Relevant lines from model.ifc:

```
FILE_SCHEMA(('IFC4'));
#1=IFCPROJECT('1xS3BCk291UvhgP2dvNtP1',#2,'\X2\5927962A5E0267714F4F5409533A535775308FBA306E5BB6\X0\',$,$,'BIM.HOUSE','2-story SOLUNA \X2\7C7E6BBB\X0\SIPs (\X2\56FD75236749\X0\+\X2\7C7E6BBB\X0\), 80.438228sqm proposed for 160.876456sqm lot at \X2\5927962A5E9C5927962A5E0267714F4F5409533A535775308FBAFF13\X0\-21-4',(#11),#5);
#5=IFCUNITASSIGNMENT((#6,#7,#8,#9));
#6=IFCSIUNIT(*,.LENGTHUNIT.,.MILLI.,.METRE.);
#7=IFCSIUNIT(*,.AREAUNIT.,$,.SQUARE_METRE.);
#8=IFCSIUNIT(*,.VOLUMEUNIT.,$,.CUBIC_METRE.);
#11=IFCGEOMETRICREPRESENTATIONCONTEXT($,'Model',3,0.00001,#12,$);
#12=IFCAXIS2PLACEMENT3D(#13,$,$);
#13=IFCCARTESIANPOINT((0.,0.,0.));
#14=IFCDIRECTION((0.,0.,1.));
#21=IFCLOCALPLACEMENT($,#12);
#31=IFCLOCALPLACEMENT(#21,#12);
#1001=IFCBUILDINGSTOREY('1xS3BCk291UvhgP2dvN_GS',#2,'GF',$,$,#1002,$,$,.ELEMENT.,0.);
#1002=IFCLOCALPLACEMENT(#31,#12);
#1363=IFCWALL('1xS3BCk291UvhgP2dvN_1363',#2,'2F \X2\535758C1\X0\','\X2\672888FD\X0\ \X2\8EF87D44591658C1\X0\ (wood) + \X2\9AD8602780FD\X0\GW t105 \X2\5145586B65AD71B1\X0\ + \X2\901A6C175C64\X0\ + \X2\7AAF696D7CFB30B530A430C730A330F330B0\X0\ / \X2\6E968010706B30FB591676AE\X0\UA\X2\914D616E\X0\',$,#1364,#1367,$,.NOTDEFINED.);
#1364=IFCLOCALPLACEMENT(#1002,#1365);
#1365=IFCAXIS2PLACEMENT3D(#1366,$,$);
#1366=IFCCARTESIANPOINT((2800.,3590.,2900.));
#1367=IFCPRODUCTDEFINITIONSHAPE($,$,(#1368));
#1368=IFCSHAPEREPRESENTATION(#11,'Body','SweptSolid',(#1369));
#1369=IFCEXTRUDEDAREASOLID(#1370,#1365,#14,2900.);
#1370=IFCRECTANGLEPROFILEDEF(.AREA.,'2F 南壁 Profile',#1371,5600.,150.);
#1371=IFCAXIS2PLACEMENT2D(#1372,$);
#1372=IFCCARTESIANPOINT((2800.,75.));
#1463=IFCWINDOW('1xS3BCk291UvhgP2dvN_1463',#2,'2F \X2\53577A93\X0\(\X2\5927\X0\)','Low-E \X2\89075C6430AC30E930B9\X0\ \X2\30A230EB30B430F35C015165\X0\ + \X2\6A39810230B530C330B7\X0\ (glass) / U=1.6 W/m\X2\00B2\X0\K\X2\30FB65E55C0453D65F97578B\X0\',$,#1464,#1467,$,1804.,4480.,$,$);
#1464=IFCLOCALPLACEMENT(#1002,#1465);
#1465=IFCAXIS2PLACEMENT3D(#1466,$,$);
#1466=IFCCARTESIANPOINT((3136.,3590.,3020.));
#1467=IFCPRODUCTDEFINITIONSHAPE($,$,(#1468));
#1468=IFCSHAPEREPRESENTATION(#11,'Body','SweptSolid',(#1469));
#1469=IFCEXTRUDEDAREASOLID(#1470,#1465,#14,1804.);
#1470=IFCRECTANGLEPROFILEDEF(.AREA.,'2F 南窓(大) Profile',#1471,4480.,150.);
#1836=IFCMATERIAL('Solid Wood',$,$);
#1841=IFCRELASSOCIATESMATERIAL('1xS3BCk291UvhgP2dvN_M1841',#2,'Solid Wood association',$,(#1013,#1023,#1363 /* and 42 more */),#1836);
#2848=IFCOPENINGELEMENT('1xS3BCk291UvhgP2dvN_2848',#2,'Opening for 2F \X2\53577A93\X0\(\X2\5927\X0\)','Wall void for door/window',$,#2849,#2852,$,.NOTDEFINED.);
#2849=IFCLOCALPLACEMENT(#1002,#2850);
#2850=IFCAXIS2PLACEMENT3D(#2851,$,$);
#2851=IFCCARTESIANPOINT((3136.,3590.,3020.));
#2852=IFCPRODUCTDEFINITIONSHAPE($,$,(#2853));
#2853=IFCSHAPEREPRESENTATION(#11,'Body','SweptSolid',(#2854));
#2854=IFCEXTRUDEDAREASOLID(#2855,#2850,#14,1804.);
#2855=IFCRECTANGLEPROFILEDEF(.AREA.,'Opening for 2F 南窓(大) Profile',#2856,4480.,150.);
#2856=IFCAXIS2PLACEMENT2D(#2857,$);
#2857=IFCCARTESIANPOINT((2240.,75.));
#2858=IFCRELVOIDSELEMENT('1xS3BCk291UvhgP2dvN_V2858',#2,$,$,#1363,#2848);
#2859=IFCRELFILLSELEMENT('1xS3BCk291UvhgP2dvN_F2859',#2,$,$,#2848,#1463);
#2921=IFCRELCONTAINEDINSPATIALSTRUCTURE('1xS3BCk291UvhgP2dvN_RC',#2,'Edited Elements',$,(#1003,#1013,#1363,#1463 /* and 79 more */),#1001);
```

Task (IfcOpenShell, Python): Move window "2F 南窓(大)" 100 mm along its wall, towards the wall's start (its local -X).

```python
import ifcopenshell
import ifcopenshell.api.geometry
import ifcopenshell.util.placement
import ifcopenshell.util.unit

model = ifcopenshell.open("model.ifc")
unit_scale = ifcopenshell.util.unit.calculate_unit_scale(model)

window = model.by_guid("1xS3BCk291UvhgP2dvN_1463")
opening = window.FillsVoids[0].RelatingOpeningElement
wall = opening.VoidsElements[0].RelatingBuildingElement

wall_matrix = ifcopenshell.util.placement.get_local_placement(wall.ObjectPlacement)
shift = wall_matrix[:3, 0] * -0.1 / unit_scale
before = ifcopenshell.util.placement.get_local_placement(window.ObjectPlacement)[:3, 3].copy()

# The window is not placed relative to its opening, so move both.
for product in (opening, window):
    matrix = ifcopenshell.util.placement.get_local_placement(product.ObjectPlacement)
    matrix[:3, 3] += shift
    ifcopenshell.api.geometry.edit_object_placement(model, product=product, matrix=matrix, is_si=False)

after = ifcopenshell.util.placement.get_local_placement(window.ObjectPlacement)[:3, 3]
print("window moved by", (after - before).round(3) + 0.0)

model.write("model_edited.ifc")
```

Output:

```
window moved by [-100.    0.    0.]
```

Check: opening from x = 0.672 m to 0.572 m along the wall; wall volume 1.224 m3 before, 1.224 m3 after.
